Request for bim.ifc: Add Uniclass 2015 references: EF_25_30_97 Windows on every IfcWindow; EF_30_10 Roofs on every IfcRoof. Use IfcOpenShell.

First a look at what the model holds.

```python
import ifcopenshell

model = ifcopenshell.open("bim.ifc")
print(model.schema)
print("classifications:", [c.Name for c in model.by_type("IfcClassification")])
for ifc_class in ("IfcDoor", "IfcRoof", "IfcStair", "IfcWall", "IfcWindow"):
    print(ifc_class, len(model.by_type(ifc_class)))
```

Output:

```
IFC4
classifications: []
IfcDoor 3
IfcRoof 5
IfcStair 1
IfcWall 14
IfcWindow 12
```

```python
import ifcopenshell
import ifcopenshell.api.classification

model = ifcopenshell.open("bim.ifc")

system = ifcopenshell.api.classification.add_classification(model, classification="Uniclass 2015")

codes = {
    "IfcWindow": ("EF_25_30_97", "Windows"),
    "IfcRoof": ("EF_30_10", "Roofs"),
}
for ifc_class, (code, name) in codes.items():
    products = model.by_type(ifc_class)
    ifcopenshell.api.classification.add_reference(
        model, products=products, classification=system, identification=code, name=name
    )
    print(code, len(products))

model.write("bim_updated.ifc")
```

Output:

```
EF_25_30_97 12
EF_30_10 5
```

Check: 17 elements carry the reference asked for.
